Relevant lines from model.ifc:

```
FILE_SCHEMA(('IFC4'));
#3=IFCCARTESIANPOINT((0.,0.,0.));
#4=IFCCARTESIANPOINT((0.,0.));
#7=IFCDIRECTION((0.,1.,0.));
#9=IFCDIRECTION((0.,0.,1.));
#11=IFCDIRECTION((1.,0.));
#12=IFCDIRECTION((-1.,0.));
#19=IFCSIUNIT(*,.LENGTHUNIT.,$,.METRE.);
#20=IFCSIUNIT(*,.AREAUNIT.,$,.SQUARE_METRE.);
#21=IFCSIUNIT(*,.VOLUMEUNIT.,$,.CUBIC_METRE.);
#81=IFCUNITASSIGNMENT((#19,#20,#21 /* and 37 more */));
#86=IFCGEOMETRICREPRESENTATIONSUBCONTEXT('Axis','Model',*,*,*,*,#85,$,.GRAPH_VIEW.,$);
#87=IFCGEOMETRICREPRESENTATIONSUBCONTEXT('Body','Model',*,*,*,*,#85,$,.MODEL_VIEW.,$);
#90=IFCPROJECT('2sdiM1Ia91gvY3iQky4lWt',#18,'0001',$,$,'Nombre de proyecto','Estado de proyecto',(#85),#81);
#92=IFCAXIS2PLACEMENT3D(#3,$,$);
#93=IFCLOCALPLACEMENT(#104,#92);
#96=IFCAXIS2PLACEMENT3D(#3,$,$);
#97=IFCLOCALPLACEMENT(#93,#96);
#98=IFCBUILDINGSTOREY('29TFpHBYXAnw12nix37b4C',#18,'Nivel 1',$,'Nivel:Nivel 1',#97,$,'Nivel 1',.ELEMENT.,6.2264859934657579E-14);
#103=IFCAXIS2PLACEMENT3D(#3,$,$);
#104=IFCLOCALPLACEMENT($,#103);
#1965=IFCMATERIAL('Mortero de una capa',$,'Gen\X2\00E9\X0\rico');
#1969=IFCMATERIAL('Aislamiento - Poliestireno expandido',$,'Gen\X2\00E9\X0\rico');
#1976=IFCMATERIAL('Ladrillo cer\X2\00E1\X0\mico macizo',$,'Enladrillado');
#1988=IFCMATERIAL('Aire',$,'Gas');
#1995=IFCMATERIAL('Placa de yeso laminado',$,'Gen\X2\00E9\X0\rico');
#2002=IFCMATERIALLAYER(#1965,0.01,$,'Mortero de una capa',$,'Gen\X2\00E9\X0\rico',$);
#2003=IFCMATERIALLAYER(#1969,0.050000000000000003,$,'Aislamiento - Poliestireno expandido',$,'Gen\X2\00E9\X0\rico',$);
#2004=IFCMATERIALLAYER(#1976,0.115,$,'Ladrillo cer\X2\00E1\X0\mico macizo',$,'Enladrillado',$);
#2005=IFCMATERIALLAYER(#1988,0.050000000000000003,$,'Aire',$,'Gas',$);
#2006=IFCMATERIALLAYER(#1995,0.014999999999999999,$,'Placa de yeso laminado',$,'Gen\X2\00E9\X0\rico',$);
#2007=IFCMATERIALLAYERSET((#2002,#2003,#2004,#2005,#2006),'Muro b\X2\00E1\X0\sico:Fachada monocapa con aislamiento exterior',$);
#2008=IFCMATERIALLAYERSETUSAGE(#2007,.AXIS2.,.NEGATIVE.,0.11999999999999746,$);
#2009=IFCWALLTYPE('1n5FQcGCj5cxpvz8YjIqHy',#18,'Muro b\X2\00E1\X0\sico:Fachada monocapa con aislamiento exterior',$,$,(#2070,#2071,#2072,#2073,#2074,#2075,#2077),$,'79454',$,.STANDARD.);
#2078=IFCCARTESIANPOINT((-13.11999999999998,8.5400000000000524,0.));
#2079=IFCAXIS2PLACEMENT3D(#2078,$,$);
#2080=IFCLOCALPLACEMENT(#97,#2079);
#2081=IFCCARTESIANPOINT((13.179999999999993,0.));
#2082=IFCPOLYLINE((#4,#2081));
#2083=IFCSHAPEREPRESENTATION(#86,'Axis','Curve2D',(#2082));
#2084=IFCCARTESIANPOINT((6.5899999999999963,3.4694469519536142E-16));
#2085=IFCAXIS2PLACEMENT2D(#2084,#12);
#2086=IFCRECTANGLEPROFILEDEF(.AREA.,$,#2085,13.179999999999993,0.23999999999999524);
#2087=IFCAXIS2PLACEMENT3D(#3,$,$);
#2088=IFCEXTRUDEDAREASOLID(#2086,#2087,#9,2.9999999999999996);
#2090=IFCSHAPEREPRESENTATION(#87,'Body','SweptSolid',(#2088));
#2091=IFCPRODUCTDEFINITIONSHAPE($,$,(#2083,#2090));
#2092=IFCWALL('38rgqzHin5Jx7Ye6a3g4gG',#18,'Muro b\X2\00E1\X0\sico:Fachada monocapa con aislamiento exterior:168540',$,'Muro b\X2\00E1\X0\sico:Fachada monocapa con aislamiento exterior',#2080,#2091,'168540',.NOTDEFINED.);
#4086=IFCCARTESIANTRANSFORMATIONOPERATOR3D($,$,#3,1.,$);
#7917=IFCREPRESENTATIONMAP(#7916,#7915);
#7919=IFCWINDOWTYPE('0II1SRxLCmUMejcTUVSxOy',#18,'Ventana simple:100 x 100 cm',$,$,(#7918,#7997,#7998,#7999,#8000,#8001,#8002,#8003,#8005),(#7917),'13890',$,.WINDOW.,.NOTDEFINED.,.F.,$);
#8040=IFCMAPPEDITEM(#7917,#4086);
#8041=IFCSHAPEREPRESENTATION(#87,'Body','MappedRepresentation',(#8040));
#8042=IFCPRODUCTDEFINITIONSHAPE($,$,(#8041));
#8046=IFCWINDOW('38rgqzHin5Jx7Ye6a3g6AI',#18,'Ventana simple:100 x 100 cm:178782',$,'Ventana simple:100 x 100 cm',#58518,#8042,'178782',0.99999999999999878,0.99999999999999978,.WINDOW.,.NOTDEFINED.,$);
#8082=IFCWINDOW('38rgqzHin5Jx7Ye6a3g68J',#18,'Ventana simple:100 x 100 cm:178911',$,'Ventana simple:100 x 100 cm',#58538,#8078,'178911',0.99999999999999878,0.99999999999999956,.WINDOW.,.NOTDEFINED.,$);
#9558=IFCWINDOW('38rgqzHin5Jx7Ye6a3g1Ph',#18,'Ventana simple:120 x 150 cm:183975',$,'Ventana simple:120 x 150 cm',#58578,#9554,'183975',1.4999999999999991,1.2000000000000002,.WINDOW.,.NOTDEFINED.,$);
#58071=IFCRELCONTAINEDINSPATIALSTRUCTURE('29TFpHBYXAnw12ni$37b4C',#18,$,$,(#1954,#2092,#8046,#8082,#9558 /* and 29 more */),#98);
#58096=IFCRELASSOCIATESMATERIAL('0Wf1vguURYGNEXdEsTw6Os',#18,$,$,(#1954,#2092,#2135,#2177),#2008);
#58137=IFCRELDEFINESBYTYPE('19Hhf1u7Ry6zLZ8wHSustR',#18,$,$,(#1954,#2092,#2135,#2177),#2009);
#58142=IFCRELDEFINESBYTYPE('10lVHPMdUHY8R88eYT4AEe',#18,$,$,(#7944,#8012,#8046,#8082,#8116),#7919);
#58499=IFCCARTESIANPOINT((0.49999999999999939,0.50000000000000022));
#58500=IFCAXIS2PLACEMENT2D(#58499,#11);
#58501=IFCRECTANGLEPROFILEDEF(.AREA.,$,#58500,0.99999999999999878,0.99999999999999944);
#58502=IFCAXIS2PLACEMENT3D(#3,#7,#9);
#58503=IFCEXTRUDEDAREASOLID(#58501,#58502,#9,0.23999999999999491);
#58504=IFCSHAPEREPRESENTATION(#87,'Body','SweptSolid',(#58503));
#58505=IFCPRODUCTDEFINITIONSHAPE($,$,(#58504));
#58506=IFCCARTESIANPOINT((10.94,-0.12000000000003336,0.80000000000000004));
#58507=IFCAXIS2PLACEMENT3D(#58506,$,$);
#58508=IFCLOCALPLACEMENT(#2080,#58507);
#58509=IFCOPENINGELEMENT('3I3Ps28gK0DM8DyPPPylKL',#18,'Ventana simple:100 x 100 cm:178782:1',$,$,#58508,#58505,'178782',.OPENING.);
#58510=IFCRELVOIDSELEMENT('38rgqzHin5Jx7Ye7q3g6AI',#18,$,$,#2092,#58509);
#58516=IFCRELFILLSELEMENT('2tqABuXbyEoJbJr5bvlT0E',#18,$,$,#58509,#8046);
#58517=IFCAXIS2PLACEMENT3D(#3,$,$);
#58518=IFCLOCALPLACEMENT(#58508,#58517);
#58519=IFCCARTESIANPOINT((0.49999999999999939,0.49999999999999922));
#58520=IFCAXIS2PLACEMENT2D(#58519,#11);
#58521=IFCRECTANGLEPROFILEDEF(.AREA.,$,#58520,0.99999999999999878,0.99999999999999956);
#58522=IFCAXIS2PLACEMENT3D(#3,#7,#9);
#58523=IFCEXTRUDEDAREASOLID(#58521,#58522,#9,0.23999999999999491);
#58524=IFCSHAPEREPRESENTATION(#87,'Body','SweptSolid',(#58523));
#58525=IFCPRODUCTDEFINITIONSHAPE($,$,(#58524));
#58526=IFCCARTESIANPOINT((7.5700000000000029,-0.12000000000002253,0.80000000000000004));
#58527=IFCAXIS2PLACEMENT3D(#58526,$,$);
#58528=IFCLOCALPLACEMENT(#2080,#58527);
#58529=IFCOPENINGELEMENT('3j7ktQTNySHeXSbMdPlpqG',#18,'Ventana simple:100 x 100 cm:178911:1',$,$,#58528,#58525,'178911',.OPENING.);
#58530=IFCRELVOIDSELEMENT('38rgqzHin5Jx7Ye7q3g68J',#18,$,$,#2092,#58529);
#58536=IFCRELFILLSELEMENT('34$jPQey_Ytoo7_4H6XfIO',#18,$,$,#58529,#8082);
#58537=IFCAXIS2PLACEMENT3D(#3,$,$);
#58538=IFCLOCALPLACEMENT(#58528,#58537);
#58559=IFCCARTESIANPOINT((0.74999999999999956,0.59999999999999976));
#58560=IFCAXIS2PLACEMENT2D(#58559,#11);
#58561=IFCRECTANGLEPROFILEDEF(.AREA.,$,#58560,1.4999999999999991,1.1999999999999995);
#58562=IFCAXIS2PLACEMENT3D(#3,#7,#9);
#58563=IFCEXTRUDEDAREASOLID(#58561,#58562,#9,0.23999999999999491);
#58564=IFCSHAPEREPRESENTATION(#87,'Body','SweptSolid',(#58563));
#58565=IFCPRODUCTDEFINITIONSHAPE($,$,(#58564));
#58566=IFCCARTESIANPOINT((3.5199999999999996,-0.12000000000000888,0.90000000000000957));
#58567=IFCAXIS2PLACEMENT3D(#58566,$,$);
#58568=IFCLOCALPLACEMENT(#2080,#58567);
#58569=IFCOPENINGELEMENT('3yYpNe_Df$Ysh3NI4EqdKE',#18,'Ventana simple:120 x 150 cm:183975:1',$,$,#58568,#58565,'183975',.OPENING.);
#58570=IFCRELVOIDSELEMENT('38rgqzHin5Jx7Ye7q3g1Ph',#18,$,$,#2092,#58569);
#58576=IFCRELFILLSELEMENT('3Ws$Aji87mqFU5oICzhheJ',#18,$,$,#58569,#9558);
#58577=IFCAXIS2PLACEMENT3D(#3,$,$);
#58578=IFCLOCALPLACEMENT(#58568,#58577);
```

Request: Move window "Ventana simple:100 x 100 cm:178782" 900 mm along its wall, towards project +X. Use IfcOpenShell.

```python
import ifcopenshell
import ifcopenshell.api.geometry
import ifcopenshell.util.placement
import ifcopenshell.util.unit

model = ifcopenshell.open("model.ifc")
unit_scale = ifcopenshell.util.unit.calculate_unit_scale(model)

window = model.by_id(8046)
opening = window.FillsVoids[0].RelatingOpeningElement
wall = opening.VoidsElements[0].RelatingBuildingElement

wall_matrix = ifcopenshell.util.placement.get_local_placement(wall.ObjectPlacement)
shift = wall_matrix[:3, 0] * 0.9 / unit_scale
before = ifcopenshell.util.placement.get_local_placement(window.ObjectPlacement)[:3, 3].copy()

# The window is placed relative to its opening, so it follows when the opening moves.
matrix = ifcopenshell.util.placement.get_local_placement(opening.ObjectPlacement)
matrix[:3, 3] += shift
ifcopenshell.api.geometry.edit_object_placement(
    model, product=opening, matrix=matrix, is_si=False, should_transform_children=True
)

after = ifcopenshell.util.placement.get_local_placement(window.ObjectPlacement)[:3, 3]
print("window moved by", (after - before).round(3) + 0.0)

model.write("model_v2.ifc")
```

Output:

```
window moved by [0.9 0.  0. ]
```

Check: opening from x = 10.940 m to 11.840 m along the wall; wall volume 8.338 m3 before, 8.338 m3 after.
